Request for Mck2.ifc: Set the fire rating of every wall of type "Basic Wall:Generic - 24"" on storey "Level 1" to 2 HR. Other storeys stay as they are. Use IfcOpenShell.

First a look at what the model holds.

```python
import ifcopenshell
import ifcopenshell.util.element

model = ifcopenshell.open("Mck2.ifc")
print(model.schema)
storey = next(s for s in model.by_type("IfcBuildingStorey") if s.Name == "Level 1")
walls = [e for e in ifcopenshell.util.element.get_decomposition(storey) if e.is_a("IfcWall")]
seen = {}
for e in walls:
    element_type = ifcopenshell.util.element.get_type(e)
    key = (element_type.Name if element_type != e and element_type else None, ifcopenshell.util.element.get_pset(e, "Pset_WallCommon", "FireRating"))
    seen[key] = seen.get(key, 0) + 1
for (name, value), count in sorted(seen.items(), key=str):
    print(count, "x", name, "|", value)
```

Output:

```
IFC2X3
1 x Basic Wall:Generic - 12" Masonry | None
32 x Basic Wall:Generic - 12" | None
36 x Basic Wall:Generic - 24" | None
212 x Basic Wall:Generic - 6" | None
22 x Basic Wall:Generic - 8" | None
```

```python
import ifcopenshell
import ifcopenshell.api.pset
import ifcopenshell.util.element

model = ifcopenshell.open("Mck2.ifc")

storey = next(s for s in model.by_type("IfcBuildingStorey") if s.Name == "Level 1")
walls = [e for e in ifcopenshell.util.element.get_decomposition(storey) if e.is_a("IfcWall")]

count = 0
for e in walls:
    element_type = ifcopenshell.util.element.get_type(e)
    if element_type in (None, e) or element_type.Name != 'Basic Wall:Generic - 24"':
        continue
    # add_pset returns the element's existing set when there is one.
    pset = ifcopenshell.api.pset.add_pset(model, product=e, name="Pset_WallCommon")
    ifcopenshell.api.pset.edit_pset(model, pset=pset, properties={"FireRating": "2 HR"})
    count += 1

print(count, "walls updated")

model.write("Mck2_edited.ifc")
```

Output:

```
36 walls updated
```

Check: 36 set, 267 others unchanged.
